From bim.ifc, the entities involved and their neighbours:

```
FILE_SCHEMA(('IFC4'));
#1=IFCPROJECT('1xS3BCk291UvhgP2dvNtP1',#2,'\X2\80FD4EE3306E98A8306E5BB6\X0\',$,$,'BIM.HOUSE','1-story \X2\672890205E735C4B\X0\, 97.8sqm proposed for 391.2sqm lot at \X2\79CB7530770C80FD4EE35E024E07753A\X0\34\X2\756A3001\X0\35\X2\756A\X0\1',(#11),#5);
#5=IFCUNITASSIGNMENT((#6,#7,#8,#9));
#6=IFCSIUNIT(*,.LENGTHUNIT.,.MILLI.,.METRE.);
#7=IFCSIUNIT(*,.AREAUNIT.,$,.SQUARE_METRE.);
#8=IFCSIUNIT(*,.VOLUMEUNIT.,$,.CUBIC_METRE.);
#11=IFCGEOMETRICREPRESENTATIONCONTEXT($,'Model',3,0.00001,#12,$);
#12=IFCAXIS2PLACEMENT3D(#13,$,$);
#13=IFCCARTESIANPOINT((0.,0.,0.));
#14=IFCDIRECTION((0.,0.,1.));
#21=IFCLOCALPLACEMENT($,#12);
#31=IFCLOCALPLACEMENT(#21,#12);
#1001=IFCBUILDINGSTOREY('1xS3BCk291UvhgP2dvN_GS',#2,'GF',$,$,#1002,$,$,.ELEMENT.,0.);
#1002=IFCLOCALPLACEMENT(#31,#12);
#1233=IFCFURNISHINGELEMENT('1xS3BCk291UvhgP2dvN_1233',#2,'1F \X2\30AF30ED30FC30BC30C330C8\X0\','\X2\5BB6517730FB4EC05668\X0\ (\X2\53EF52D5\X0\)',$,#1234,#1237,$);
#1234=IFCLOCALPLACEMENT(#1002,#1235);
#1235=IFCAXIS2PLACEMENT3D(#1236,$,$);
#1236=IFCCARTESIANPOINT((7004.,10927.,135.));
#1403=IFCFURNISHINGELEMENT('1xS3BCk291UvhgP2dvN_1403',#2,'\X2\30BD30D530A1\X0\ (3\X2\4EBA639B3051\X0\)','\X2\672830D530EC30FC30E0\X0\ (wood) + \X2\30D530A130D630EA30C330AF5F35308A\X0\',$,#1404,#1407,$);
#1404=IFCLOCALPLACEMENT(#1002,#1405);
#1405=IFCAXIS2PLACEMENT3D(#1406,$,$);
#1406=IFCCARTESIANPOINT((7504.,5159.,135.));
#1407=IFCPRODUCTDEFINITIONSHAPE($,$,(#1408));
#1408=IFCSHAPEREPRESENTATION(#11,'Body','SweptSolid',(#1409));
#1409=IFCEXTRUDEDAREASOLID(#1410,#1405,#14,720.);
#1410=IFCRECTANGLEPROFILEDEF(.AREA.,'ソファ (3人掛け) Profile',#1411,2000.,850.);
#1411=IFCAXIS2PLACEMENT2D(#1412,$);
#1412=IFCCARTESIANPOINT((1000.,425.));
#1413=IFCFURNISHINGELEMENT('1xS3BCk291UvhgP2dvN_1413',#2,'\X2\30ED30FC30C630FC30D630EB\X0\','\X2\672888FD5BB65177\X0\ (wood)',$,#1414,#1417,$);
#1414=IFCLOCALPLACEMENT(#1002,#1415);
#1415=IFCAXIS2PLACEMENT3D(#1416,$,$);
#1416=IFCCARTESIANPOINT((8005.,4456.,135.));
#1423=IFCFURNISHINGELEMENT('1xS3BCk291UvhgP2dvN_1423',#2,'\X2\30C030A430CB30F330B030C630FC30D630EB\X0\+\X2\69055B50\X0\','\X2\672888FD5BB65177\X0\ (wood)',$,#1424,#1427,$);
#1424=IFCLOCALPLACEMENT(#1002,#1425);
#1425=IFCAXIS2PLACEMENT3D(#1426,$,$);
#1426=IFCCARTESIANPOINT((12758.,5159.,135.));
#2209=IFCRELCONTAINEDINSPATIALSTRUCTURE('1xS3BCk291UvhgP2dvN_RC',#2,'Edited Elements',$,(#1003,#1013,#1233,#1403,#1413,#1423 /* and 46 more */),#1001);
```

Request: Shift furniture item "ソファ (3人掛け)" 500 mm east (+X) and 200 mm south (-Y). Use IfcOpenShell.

```python
import ifcopenshell
import ifcopenshell.api.geometry
import ifcopenshell.util.placement
import ifcopenshell.util.unit

model = ifcopenshell.open("bim.ifc")
unit_scale = ifcopenshell.util.unit.calculate_unit_scale(model)

item = model.by_guid("1xS3BCk291UvhgP2dvN_1403")
matrix = ifcopenshell.util.placement.get_local_placement(item.ObjectPlacement)
matrix[0, 3] += 0.5 / unit_scale
matrix[1, 3] -= 0.2 / unit_scale
ifcopenshell.api.geometry.edit_object_placement(model, product=item, matrix=matrix, is_si=False)

print(ifcopenshell.util.placement.get_local_placement(item.ObjectPlacement).round(3) + 0.0)

model.write("bim_edited.ifc")
```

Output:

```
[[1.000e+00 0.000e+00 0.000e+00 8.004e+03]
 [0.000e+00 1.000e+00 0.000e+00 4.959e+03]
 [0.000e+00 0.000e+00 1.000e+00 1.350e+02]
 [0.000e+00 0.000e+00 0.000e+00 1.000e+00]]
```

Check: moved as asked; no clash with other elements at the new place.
